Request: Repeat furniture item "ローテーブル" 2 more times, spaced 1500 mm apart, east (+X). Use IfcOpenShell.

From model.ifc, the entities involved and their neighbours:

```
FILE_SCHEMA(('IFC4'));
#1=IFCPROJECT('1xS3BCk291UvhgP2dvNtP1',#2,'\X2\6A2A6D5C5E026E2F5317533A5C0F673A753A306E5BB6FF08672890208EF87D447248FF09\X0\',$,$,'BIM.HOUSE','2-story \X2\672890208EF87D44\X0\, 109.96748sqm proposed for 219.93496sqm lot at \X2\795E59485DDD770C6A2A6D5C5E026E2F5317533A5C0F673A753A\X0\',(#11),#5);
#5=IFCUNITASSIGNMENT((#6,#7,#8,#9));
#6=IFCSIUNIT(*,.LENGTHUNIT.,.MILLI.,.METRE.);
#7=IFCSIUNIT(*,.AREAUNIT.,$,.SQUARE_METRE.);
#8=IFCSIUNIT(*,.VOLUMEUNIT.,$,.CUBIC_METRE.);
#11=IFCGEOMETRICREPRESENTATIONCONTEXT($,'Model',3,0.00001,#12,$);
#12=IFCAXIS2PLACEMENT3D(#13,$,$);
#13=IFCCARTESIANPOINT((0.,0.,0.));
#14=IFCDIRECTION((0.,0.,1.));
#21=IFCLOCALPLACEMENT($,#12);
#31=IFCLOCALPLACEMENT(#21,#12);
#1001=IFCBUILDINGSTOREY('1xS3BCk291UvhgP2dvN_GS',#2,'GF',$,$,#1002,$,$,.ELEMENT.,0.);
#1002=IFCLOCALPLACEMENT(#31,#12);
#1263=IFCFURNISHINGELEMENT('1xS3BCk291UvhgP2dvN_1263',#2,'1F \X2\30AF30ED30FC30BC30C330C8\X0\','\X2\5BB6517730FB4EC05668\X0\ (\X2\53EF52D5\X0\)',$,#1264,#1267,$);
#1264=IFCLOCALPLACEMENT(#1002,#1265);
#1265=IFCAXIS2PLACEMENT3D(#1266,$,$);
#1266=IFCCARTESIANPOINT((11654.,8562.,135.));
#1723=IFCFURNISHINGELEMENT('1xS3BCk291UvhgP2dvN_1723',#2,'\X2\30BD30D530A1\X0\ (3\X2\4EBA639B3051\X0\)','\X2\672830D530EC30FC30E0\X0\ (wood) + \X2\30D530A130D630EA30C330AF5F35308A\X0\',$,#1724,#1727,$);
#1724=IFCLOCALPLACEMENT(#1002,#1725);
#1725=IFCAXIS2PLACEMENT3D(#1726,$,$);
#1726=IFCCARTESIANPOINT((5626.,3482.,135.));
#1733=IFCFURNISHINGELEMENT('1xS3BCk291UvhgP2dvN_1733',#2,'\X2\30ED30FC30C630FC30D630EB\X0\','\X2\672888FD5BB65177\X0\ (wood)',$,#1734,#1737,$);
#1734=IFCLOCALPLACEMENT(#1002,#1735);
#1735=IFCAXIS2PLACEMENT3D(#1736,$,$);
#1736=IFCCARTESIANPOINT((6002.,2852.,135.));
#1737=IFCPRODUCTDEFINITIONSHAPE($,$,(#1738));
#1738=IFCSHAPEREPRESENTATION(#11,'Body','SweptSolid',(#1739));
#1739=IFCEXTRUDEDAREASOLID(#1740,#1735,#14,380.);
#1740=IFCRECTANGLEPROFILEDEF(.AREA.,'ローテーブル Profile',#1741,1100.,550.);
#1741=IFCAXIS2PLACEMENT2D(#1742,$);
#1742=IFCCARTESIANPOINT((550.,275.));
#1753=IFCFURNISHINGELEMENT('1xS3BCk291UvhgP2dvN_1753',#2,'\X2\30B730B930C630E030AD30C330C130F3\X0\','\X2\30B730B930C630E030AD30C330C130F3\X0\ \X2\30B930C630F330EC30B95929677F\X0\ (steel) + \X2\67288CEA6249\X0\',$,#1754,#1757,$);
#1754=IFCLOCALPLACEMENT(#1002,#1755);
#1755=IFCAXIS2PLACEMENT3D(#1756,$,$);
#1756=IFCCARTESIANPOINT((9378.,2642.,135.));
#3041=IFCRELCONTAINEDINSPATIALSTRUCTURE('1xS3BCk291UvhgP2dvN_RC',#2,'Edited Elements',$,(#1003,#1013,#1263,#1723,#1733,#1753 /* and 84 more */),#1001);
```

```python
import numpy as np
import ifcopenshell
import ifcopenshell.api.geometry
import ifcopenshell.api.root
import ifcopenshell.util.element
import ifcopenshell.util.placement
import ifcopenshell.util.unit

model = ifcopenshell.open("model.ifc")
unit_scale = ifcopenshell.util.unit.calculate_unit_scale(model)


def reuse_history(source, copy):
    """copy_class also copies each property set's owner history, people and application; keep the originals."""
    for rel in copy.IsDefinedBy:
        if rel.is_a("IfcRelDefinesByProperties") and (history := rel.RelatingPropertyDefinition.OwnerHistory):
            rel.RelatingPropertyDefinition.OwnerHistory = source.OwnerHistory
            ifcopenshell.util.element.remove_deep2(model, history)


source = model.by_guid("1xS3BCk291UvhgP2dvN_1733")
base = ifcopenshell.util.placement.get_local_placement(source.ObjectPlacement)
step = np.array([1.0, 0.0, 0.0]) * 1.5 / unit_scale

for i in range(1, 3):
    copy = ifcopenshell.api.root.copy_class(model, product=source)
    copy.Representation = ifcopenshell.util.element.copy_deep(
        model, source.Representation, exclude=["IfcGeometricRepresentationContext", "IfcRepresentationMap"]
    )
    reuse_history(source, copy)
    matrix = base.copy()
    matrix[:3, 3] += i * step
    print("added at", matrix[:3, 3].round(3) + 0.0)
    ifcopenshell.api.geometry.edit_object_placement(model, product=copy, matrix=matrix, is_si=False)

model.write("model-out.ifc")
```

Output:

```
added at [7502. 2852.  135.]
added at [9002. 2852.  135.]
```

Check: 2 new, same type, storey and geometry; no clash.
